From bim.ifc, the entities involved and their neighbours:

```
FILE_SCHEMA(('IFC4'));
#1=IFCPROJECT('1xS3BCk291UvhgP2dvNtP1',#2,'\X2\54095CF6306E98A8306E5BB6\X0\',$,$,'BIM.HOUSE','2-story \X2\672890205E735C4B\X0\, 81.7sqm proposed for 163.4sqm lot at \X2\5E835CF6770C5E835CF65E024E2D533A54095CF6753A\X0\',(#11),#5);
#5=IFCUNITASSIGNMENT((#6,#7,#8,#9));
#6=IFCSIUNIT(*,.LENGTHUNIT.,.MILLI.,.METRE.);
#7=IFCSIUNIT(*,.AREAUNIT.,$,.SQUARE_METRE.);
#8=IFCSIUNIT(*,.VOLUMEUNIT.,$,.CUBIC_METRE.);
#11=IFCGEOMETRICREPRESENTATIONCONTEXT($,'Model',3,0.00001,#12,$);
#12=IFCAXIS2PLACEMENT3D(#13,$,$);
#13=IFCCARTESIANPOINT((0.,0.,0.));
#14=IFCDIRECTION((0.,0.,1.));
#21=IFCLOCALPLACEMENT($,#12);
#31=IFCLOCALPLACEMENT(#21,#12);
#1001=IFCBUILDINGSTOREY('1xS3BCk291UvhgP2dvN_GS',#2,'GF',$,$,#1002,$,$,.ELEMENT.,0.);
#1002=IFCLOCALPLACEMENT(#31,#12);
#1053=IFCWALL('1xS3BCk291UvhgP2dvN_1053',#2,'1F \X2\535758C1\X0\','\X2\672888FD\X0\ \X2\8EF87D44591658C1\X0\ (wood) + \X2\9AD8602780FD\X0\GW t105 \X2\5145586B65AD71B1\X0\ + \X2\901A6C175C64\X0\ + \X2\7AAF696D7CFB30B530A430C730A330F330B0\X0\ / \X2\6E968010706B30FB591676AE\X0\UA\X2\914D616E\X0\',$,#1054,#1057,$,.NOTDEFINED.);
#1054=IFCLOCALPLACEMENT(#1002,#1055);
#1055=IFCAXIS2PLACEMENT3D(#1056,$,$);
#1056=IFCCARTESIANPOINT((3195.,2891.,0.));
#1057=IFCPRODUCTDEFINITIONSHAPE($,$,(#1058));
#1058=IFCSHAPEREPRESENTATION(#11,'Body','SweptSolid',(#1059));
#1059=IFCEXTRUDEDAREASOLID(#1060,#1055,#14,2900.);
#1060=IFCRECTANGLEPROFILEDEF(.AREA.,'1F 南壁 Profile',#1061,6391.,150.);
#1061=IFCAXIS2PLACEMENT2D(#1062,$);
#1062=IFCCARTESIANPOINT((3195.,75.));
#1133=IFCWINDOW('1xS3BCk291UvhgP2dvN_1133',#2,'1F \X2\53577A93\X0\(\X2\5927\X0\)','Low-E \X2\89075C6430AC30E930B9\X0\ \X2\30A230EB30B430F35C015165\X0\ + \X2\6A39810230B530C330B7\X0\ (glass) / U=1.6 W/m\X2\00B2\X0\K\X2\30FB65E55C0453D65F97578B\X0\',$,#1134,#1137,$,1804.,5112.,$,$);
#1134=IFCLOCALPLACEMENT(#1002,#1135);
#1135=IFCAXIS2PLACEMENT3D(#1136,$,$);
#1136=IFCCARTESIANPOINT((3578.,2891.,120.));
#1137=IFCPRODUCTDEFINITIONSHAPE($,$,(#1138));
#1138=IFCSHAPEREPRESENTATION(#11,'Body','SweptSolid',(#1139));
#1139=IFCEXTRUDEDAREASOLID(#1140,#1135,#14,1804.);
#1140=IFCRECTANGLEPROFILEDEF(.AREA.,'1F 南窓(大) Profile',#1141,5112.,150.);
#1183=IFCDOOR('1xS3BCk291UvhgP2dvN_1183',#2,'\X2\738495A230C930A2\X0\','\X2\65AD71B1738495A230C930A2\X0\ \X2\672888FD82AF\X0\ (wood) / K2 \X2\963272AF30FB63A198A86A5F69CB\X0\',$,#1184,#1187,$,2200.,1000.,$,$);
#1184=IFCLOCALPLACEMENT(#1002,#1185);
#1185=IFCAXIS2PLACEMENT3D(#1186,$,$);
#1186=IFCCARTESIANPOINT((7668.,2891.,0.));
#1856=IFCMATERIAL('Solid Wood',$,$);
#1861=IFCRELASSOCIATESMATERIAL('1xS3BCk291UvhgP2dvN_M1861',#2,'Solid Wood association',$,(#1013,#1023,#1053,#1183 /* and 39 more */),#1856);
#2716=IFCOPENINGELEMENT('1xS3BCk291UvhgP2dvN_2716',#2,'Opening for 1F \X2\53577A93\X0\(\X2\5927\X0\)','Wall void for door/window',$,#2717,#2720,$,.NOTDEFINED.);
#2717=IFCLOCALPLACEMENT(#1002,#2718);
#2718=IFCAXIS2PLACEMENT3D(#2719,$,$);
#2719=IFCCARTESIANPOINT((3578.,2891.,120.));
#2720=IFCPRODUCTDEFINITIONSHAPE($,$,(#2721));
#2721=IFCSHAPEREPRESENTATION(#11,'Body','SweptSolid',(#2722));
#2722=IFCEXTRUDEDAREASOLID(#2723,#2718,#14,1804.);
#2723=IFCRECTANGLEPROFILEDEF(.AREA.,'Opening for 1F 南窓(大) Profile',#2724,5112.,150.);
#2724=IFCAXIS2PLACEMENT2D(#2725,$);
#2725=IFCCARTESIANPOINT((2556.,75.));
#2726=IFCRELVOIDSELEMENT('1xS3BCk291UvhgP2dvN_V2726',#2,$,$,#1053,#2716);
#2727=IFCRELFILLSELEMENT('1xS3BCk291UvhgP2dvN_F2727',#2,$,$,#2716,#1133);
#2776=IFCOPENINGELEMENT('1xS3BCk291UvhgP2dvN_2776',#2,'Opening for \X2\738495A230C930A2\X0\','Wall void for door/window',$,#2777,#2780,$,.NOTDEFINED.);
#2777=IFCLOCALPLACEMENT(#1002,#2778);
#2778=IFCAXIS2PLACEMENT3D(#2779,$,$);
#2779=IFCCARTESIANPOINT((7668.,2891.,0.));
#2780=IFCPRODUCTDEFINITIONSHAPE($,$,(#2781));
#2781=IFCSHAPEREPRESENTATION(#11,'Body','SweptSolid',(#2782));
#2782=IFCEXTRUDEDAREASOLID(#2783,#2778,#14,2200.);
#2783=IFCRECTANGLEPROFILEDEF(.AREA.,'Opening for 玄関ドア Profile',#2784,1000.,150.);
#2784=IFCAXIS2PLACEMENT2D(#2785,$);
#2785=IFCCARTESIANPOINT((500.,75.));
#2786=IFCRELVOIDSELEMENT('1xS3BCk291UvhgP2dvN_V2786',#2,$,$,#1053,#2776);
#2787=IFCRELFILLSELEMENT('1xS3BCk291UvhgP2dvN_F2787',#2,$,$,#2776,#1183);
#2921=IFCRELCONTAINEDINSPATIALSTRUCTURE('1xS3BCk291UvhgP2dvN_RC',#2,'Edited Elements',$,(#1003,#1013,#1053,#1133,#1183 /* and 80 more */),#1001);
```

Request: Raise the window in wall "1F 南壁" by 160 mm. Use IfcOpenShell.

```python
import numpy as np
import ifcopenshell
import ifcopenshell.api.geometry
import ifcopenshell.util.placement
import ifcopenshell.util.unit

model = ifcopenshell.open("bim.ifc")
unit_scale = ifcopenshell.util.unit.calculate_unit_scale(model)

window = model.by_guid("1xS3BCk291UvhgP2dvN_1133")
opening = window.FillsVoids[0].RelatingOpeningElement
dz = 0.16 / unit_scale

shift = np.array([0.0, 0.0, dz])
# The window is not placed relative to its opening, so move both.
for product in (opening, window):
    matrix = ifcopenshell.util.placement.get_local_placement(product.ObjectPlacement)
    matrix[:3, 3] += shift
    ifcopenshell.api.geometry.edit_object_placement(model, product=product, matrix=matrix, is_si=False)

print(f"moved by {dz * unit_scale:+.3f} m")

model.write("bim_updated.ifc")
```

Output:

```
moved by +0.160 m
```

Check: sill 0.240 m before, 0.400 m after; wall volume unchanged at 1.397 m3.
